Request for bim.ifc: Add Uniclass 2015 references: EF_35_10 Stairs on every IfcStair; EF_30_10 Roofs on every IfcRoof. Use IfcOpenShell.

First a look at what the model holds.

```python
import ifcopenshell

model = ifcopenshell.open("bim.ifc")
print(model.schema)
print("classifications:", [c.Name for c in model.by_type("IfcClassification")])
for ifc_class in ("IfcDoor", "IfcRoof", "IfcStair", "IfcWall", "IfcWindow"):
    print(ifc_class, len(model.by_type(ifc_class)))
```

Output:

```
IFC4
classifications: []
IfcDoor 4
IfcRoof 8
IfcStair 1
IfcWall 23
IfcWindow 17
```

```python
import ifcopenshell
import ifcopenshell.api.classification

model = ifcopenshell.open("bim.ifc")

system = ifcopenshell.api.classification.add_classification(model, classification="Uniclass 2015")

codes = {
    "IfcStair": ("EF_35_10", "Stairs"),
    "IfcRoof": ("EF_30_10", "Roofs"),
}
for ifc_class, (code, name) in codes.items():
    products = model.by_type(ifc_class)
    ifcopenshell.api.classification.add_reference(
        model, products=products, classification=system, identification=code, name=name
    )
    print(code, len(products))

model.write("bim_rev.ifc")
```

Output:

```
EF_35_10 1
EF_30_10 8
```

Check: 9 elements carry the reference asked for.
